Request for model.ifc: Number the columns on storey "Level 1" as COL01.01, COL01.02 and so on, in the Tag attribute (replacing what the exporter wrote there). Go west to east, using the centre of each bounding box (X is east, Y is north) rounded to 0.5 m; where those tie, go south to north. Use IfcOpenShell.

First a look at what the model holds.

```python
import ifcopenshell
import ifcopenshell.util.element
import ifcopenshell.util.placement

model = ifcopenshell.open("model.ifc")
print(model.schema)
storey = next(s for s in model.by_type("IfcBuildingStorey") if s.Name == "Level 1")
columns = [e for e in ifcopenshell.util.element.get_decomposition(storey) if e.is_a("IfcColumn")]
for e in sorted(columns, key=lambda e: e.id()):
    origin = ifcopenshell.util.placement.get_local_placement(e.ObjectPlacement)[:3, 3]
    print(e.id(), e.Tag, e.Name, origin.round(2) + 0.0, sep=" | ")
```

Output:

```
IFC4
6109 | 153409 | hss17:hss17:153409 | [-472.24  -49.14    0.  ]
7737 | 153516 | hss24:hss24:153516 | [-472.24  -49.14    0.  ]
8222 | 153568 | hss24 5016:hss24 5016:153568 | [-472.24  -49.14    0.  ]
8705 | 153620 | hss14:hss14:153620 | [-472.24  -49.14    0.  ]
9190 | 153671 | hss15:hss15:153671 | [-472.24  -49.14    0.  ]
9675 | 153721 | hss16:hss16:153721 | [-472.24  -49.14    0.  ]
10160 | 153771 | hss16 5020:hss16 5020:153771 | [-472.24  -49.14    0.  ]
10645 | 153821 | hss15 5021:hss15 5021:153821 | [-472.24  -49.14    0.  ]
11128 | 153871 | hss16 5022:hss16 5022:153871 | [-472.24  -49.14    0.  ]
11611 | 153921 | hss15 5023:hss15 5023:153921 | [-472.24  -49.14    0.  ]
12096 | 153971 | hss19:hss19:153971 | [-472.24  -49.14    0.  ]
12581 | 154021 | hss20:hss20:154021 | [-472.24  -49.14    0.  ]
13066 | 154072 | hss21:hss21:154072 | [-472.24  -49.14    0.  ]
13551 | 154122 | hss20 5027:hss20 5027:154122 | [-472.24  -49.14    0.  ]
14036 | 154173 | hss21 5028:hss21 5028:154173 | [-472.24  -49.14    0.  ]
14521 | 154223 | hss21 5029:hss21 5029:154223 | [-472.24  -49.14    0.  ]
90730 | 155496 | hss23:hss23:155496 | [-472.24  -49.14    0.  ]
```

```python
import ifcopenshell
import ifcopenshell.geom
import ifcopenshell.util.element
import ifcopenshell.util.shape

model = ifcopenshell.open("model.ifc")
settings = ifcopenshell.geom.settings()
settings.set("use-world-coords", True)


def centre(element):
    shape = ifcopenshell.geom.create_shape(settings, element)
    return ifcopenshell.util.shape.get_bbox_centroid(shape.geometry)


storey = next(s for s in model.by_type("IfcBuildingStorey") if s.Name == "Level 1")
columns = [e for e in ifcopenshell.util.element.get_decomposition(storey) if e.is_a("IfcColumn")]

# Insertion points can sit at a corner or the storey origin, so sort by the geometry (in metres).
centres = {e: centre(e) for e in columns}
columns.sort(key=lambda e: (round(centres[e][0] / 0.5), centres[e][1]))

for i, e in enumerate(columns, start=1):
    number = f"COL01.{i:02d}"
    e.Tag = number
    print(e.id(), number)

model.write("model_v2.ifc")
```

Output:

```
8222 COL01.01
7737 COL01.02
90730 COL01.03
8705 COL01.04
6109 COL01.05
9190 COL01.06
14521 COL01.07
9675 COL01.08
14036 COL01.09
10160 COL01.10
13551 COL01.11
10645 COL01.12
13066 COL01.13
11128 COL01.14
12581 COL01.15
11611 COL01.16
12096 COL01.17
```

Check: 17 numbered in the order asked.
